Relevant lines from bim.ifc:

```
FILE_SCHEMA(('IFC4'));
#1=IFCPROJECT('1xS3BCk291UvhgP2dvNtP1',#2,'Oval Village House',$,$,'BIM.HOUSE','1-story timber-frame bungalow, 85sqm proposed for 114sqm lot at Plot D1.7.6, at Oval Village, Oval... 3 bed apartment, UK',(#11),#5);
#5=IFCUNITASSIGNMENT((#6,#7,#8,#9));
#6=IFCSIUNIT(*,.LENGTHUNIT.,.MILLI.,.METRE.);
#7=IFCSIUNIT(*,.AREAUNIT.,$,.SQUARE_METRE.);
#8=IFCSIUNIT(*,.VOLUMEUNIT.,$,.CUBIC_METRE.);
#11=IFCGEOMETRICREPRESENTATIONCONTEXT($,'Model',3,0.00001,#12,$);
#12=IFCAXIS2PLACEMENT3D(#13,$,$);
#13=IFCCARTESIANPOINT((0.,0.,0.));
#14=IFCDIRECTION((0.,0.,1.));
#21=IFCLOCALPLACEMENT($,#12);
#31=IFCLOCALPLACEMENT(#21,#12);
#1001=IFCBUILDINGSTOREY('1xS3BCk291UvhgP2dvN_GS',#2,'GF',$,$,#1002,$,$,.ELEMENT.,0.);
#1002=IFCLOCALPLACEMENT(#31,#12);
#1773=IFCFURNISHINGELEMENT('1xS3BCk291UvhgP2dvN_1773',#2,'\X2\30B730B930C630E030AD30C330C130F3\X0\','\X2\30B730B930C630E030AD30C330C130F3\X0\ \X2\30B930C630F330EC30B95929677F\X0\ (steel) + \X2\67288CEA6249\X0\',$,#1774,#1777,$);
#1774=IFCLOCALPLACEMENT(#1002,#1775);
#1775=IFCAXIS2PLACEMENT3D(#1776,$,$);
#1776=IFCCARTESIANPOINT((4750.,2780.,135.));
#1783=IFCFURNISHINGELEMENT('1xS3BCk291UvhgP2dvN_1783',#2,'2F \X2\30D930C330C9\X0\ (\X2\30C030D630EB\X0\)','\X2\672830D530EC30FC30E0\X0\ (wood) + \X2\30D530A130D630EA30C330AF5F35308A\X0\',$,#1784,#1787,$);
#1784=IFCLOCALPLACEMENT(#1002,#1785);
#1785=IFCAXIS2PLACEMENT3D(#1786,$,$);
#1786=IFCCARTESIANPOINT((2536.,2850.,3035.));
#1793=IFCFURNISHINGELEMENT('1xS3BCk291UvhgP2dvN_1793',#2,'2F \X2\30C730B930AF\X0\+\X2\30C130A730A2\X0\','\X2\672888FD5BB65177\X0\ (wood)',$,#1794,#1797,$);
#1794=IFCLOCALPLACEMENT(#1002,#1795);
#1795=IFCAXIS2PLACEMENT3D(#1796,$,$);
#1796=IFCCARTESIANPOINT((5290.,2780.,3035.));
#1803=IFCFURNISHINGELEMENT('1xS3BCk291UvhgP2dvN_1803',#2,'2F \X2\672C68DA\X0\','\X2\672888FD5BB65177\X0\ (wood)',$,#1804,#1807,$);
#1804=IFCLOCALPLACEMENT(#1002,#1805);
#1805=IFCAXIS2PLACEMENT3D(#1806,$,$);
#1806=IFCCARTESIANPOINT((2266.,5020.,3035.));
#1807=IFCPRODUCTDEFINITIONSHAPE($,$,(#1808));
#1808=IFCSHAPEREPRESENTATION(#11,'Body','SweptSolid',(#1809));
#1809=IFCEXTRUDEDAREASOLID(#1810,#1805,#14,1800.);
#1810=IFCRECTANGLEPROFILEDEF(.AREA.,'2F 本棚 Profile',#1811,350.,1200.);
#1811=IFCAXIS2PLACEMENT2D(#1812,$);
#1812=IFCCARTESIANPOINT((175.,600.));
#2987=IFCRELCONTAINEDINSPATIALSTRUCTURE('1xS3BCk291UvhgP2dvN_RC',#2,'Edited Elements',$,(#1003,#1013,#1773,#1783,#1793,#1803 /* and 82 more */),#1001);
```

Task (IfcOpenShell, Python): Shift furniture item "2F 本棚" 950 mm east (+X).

```python
import ifcopenshell
import ifcopenshell.api.geometry
import ifcopenshell.util.placement
import ifcopenshell.util.unit

model = ifcopenshell.open("bim.ifc")
unit_scale = ifcopenshell.util.unit.calculate_unit_scale(model)

item = model.by_guid("1xS3BCk291UvhgP2dvN_1803")
matrix = ifcopenshell.util.placement.get_local_placement(item.ObjectPlacement)
matrix[0, 3] += 0.95 / unit_scale
ifcopenshell.api.geometry.edit_object_placement(model, product=item, matrix=matrix, is_si=False)

print(ifcopenshell.util.placement.get_local_placement(item.ObjectPlacement).round(3) + 0.0)

model.write("bim_v2.ifc")
```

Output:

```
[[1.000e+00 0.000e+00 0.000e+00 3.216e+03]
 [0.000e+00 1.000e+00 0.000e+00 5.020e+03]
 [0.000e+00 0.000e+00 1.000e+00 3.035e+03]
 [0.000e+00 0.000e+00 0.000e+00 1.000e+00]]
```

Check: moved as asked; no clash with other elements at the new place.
